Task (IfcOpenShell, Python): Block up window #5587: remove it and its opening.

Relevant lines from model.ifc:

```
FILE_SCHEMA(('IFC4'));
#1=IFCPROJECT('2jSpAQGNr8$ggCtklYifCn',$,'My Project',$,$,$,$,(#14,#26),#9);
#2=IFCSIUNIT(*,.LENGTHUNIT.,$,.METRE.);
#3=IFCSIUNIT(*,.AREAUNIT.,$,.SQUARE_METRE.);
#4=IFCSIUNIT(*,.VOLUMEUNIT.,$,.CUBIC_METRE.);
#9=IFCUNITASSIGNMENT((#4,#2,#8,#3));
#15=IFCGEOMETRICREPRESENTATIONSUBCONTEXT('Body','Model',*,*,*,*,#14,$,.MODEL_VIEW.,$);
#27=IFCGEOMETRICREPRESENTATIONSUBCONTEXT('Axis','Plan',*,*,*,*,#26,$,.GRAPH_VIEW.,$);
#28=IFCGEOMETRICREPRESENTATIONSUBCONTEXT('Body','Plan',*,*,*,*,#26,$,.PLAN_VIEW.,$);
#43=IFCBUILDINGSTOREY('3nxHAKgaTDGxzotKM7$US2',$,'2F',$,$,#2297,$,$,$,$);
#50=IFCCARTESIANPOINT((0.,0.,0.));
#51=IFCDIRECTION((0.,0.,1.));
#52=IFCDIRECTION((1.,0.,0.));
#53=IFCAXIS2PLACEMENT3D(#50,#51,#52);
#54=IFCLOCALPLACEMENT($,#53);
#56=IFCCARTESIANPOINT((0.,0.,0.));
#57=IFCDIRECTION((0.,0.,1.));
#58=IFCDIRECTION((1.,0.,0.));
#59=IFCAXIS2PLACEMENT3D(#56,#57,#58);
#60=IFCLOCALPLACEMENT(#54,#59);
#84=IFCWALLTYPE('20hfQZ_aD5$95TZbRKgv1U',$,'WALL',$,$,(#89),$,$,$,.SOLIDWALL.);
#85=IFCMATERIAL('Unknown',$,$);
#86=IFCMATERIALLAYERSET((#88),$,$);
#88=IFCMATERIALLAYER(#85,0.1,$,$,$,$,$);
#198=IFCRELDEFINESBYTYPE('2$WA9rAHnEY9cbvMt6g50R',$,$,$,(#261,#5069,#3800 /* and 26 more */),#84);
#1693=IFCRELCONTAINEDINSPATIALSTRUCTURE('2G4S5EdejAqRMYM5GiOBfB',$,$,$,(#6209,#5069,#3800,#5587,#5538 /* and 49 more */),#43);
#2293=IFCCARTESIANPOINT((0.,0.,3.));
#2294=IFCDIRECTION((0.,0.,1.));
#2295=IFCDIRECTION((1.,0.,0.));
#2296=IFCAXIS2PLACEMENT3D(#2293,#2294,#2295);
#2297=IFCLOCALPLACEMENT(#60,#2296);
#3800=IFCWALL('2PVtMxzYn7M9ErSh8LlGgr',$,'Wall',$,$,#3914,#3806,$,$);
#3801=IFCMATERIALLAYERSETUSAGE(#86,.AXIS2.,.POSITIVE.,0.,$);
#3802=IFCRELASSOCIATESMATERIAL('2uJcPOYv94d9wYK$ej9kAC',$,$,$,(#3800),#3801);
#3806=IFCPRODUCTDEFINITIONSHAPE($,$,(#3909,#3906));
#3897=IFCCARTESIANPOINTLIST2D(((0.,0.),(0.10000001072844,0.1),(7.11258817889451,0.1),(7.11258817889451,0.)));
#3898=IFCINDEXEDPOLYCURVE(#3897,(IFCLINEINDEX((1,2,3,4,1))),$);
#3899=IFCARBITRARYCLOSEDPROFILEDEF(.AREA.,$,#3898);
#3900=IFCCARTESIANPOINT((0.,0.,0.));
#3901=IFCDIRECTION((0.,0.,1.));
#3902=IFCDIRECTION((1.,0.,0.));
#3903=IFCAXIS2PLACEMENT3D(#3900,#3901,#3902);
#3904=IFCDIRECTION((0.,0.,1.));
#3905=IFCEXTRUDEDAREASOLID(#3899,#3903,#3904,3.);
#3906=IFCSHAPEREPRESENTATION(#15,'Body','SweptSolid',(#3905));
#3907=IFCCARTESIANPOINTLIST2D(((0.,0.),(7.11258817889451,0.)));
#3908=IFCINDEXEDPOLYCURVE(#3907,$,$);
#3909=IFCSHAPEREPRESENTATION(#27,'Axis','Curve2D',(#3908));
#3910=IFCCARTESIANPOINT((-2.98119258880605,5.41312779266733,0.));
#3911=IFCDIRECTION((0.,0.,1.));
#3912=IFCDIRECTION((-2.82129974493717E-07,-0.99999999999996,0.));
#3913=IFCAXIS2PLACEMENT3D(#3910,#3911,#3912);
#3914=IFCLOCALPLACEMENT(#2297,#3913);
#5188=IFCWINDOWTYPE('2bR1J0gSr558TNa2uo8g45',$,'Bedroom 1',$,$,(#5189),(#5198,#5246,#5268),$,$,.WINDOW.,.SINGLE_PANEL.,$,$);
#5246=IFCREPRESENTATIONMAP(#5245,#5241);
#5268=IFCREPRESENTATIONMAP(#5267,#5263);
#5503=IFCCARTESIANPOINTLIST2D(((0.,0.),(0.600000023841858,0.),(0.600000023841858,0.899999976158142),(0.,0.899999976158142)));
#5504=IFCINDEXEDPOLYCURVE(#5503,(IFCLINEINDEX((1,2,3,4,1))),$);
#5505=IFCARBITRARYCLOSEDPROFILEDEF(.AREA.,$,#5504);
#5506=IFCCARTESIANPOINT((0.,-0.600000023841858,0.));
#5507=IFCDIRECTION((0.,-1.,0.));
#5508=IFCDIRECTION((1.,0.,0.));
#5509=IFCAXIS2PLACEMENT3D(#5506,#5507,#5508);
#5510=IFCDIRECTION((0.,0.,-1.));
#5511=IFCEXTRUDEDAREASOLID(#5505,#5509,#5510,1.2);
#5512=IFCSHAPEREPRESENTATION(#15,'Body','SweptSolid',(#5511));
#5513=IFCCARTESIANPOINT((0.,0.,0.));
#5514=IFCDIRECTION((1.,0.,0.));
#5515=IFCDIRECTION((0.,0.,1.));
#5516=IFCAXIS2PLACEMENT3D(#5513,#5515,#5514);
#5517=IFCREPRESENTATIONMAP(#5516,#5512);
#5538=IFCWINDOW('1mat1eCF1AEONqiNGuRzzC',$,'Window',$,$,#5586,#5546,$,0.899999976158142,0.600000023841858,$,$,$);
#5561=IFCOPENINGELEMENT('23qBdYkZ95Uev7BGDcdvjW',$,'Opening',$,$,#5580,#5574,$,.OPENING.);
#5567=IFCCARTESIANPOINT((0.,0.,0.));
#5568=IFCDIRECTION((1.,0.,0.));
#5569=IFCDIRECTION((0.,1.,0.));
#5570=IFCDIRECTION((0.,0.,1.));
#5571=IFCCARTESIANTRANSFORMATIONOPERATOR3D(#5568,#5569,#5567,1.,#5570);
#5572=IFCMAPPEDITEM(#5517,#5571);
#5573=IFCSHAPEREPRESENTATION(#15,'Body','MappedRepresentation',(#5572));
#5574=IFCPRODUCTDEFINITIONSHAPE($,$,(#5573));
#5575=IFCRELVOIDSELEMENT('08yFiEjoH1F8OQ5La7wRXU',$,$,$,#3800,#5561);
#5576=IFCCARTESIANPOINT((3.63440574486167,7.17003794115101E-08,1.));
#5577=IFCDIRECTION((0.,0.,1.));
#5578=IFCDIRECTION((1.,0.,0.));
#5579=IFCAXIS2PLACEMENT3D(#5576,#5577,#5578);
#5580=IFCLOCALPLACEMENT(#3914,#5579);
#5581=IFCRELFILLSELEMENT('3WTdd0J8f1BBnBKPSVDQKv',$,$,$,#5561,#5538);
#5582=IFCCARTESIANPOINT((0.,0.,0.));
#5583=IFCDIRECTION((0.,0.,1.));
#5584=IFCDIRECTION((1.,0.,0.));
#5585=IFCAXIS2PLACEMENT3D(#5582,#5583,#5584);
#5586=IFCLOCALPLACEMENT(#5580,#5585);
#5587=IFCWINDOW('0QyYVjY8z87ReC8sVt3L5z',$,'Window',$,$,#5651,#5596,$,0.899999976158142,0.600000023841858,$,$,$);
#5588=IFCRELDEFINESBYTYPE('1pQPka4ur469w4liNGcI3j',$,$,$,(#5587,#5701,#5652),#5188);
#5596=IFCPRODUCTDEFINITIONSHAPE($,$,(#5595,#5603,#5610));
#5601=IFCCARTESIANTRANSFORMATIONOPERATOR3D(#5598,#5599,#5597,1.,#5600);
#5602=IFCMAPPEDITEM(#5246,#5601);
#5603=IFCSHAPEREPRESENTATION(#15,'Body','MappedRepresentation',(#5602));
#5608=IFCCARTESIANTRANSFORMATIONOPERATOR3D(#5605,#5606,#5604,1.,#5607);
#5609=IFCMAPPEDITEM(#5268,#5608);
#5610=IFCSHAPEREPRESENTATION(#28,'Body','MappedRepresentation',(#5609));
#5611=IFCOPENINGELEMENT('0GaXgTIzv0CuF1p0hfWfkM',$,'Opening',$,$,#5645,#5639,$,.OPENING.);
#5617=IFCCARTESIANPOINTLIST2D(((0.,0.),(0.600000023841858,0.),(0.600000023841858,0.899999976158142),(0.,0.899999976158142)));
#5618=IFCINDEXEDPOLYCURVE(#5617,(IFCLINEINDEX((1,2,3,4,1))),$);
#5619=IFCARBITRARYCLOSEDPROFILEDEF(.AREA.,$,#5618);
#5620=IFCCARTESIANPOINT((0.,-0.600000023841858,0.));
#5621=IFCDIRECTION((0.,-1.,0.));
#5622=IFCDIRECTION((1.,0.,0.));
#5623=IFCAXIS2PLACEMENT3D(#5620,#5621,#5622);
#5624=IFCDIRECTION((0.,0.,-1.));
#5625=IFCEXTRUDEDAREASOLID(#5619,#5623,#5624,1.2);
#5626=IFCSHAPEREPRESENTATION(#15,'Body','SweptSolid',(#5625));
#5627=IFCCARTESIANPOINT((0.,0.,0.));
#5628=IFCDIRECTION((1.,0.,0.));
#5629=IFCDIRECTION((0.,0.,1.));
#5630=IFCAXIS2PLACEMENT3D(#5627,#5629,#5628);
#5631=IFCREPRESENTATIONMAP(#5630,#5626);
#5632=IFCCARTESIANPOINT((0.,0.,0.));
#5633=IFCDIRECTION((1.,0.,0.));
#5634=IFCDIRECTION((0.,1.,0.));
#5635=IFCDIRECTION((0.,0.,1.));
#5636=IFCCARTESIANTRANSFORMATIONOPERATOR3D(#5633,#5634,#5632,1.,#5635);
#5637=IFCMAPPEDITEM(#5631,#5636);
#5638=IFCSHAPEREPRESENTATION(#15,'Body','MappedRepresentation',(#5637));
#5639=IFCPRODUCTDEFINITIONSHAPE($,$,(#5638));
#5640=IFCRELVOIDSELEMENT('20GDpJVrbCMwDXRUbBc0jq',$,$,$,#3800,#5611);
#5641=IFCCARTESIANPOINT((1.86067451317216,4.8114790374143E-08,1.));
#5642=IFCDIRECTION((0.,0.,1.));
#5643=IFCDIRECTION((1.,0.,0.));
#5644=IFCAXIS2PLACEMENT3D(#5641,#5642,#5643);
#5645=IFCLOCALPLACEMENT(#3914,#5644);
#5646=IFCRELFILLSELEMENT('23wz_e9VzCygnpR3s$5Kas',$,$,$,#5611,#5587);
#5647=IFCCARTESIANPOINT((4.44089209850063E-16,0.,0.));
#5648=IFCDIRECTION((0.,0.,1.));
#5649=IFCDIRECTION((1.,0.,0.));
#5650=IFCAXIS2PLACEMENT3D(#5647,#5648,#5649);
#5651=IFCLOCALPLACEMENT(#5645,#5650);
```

```python
import ifcopenshell
import ifcopenshell.api.feature
import ifcopenshell.api.root
import ifcopenshell.geom
import ifcopenshell.util.shape

model = ifcopenshell.open("model.ifc")
settings = ifcopenshell.geom.settings()


def volume(element):
    """Net volume in cubic metres, openings subtracted."""
    shape = ifcopenshell.geom.create_shape(settings, element)
    return ifcopenshell.util.shape.get_volume(shape.geometry)


window = model.by_guid("0QyYVjY8z87ReC8sVt3L5z")
opening = window.FillsVoids[0].RelatingOpeningElement
wall = opening.VoidsElements[0].RelatingBuildingElement
before = volume(wall)

ifcopenshell.api.root.remove_product(model, product=window)
ifcopenshell.api.feature.remove_feature(model, feature=opening)

after = volume(wall)

print(f"wall volume {before:.3f} -> {after:.3f} m3")

model.write("model-out.ifc")
```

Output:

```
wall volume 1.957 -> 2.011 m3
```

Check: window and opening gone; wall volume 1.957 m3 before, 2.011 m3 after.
